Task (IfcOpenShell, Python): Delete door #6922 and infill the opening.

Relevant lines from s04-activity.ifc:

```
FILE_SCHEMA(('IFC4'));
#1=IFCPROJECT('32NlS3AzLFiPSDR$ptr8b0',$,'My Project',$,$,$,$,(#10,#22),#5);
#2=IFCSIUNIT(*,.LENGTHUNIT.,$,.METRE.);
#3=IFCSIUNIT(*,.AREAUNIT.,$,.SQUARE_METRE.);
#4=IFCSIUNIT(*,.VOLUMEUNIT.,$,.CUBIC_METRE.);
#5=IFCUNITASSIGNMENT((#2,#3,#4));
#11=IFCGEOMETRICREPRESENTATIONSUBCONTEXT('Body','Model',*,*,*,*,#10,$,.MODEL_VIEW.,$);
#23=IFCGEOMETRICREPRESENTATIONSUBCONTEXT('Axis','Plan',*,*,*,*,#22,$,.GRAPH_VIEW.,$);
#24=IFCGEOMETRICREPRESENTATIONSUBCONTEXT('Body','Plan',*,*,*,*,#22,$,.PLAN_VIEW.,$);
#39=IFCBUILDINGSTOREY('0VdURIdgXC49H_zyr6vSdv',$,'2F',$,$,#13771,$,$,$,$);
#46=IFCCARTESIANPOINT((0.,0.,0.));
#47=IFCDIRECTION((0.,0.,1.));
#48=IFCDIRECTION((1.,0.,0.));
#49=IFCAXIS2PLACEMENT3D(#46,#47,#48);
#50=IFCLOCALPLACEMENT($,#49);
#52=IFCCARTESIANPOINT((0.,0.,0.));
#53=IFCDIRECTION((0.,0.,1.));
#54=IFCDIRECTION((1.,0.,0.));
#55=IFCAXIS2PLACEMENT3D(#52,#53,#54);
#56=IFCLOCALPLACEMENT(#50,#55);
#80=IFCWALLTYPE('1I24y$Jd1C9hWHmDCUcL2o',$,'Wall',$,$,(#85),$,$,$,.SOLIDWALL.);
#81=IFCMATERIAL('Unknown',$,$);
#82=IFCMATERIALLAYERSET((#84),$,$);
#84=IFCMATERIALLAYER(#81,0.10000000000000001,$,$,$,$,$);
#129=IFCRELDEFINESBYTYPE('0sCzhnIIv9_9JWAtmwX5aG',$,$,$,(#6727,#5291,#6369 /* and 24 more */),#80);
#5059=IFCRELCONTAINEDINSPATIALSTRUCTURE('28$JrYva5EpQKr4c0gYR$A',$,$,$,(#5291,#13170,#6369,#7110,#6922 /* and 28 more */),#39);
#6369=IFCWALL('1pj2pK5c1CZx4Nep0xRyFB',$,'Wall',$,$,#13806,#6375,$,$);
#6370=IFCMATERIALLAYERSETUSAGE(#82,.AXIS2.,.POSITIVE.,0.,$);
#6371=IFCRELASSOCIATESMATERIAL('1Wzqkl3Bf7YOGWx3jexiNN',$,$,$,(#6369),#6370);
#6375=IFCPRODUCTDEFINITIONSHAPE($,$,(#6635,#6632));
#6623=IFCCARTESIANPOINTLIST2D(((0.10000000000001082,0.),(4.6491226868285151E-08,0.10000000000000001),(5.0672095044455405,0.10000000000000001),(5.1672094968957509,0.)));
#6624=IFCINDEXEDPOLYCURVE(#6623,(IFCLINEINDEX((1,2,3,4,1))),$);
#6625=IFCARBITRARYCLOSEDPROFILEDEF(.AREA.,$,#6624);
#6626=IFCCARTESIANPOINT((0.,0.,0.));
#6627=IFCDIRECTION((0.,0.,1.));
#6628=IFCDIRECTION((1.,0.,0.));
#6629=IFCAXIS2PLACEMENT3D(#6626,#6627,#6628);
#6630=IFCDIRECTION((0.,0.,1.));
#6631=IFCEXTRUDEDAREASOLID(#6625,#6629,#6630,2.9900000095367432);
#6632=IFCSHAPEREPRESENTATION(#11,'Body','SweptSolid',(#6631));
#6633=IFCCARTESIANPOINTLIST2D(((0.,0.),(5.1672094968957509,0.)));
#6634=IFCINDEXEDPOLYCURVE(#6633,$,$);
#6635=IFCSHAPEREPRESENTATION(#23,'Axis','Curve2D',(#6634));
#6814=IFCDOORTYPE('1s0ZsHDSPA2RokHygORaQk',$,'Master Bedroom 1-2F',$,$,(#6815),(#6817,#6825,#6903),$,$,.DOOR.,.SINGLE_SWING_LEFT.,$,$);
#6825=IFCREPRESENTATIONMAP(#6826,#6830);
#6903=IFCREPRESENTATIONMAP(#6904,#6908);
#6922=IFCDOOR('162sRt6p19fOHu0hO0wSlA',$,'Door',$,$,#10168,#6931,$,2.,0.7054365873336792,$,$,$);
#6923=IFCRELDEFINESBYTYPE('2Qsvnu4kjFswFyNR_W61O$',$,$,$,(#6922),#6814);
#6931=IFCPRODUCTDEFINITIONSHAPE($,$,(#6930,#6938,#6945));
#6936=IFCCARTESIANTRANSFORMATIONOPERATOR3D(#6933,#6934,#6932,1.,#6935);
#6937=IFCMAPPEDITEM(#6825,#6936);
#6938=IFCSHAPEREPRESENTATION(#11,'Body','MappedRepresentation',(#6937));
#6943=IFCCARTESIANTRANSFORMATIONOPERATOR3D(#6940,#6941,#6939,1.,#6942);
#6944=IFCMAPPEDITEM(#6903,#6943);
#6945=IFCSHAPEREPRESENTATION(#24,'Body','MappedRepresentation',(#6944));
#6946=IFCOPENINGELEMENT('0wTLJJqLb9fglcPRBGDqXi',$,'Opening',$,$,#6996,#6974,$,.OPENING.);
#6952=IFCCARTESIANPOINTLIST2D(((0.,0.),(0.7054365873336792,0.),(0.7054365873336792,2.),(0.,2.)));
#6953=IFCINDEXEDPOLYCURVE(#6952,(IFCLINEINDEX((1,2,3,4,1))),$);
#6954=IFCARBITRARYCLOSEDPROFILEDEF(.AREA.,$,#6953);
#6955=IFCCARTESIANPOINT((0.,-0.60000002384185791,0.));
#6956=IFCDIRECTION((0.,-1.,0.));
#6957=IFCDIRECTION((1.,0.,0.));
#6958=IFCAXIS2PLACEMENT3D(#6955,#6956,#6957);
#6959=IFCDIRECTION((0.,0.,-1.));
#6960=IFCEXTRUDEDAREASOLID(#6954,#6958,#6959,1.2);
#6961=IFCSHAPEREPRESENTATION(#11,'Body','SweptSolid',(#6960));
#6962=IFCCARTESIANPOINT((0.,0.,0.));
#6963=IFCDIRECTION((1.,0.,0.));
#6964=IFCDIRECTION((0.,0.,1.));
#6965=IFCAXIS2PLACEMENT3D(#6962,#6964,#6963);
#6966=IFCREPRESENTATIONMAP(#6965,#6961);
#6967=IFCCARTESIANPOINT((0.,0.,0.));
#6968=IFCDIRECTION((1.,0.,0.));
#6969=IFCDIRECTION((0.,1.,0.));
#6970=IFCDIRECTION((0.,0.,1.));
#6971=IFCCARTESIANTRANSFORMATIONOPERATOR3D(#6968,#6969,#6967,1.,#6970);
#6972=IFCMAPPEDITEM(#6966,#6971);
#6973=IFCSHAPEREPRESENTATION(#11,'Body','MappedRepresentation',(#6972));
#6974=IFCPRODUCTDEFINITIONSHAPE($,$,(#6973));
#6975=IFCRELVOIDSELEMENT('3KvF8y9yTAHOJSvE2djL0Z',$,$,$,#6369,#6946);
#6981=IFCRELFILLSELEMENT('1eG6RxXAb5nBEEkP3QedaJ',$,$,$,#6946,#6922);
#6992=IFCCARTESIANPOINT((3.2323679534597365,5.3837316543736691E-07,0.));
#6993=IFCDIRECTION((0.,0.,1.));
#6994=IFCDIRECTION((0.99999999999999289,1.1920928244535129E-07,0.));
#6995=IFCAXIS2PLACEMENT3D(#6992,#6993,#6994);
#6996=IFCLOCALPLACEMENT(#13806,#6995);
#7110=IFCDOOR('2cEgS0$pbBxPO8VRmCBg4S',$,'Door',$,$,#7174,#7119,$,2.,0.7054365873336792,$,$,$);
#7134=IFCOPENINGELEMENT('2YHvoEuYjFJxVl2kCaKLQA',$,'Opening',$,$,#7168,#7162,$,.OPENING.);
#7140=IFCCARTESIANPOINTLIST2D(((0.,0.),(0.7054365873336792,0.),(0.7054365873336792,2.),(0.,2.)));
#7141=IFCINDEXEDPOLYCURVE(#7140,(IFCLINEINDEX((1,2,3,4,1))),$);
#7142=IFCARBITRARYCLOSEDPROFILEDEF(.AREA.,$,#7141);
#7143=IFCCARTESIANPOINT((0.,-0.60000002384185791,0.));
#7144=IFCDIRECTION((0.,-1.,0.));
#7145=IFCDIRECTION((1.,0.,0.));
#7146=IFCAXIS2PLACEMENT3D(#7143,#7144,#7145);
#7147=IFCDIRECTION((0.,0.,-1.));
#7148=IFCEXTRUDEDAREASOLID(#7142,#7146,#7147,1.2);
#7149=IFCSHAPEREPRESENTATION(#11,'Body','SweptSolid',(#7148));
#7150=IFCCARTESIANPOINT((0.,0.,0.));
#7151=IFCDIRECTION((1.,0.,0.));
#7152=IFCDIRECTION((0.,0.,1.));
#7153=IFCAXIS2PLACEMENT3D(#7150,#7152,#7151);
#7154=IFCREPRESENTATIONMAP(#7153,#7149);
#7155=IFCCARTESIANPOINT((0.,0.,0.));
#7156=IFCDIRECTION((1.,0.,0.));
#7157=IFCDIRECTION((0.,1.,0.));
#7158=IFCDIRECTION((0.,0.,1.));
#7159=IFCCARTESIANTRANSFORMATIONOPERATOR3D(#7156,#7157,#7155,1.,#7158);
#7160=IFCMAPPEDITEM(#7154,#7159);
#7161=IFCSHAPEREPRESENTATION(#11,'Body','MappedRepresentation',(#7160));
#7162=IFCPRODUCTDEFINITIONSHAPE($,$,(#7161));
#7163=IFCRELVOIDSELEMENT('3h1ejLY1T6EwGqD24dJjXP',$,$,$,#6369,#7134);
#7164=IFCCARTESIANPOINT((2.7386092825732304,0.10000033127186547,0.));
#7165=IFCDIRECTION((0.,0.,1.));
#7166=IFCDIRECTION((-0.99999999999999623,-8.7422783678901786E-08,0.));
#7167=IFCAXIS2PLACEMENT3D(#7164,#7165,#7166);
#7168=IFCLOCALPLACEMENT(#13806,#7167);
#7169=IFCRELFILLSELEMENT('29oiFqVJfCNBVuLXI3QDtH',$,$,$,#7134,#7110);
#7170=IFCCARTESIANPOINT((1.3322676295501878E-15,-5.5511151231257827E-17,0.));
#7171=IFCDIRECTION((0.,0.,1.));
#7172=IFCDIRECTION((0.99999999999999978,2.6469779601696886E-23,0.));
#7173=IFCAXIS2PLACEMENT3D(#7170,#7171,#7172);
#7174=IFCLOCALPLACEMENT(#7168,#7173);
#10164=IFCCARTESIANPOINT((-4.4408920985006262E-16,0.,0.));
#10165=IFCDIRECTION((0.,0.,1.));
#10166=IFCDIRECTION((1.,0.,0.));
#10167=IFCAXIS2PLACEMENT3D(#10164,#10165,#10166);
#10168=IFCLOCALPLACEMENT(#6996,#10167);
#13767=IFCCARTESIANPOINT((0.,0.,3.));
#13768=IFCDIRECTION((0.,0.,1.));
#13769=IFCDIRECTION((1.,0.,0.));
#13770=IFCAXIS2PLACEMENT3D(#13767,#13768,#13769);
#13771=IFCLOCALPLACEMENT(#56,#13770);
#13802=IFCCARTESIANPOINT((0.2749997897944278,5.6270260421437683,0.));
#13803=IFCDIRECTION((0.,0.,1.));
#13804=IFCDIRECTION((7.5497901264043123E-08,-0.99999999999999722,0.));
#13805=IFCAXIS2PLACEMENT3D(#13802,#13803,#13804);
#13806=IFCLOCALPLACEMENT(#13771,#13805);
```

```python
import ifcopenshell
import ifcopenshell.api.feature
import ifcopenshell.api.root
import ifcopenshell.geom
import ifcopenshell.util.shape

model = ifcopenshell.open("s04-activity.ifc")
settings = ifcopenshell.geom.settings()


def volume(element):
    """Net volume in cubic metres, openings subtracted."""
    shape = ifcopenshell.geom.create_shape(settings, element)
    return ifcopenshell.util.shape.get_volume(shape.geometry)


door = model.by_guid("162sRt6p19fOHu0hO0wSlA")
opening = door.FillsVoids[0].RelatingOpeningElement
wall = opening.VoidsElements[0].RelatingBuildingElement
before = volume(wall)

ifcopenshell.api.root.remove_product(model, product=door)
ifcopenshell.api.feature.remove_feature(model, feature=opening)

after = volume(wall)

print(f"wall volume {before:.3f} -> {after:.3f} m3")

model.write("s04-activity_edited.ifc")
```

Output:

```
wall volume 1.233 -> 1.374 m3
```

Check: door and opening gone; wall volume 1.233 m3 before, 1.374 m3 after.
